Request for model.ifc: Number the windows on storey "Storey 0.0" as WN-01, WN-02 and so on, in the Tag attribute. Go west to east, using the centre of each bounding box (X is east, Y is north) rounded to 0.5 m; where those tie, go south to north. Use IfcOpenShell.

First a look at what the model holds.

```python
import ifcopenshell
import ifcopenshell.util.element
import ifcopenshell.util.placement

model = ifcopenshell.open("model.ifc")
print(model.schema)
storey = next(s for s in model.by_type("IfcBuildingStorey") if s.Name == "Storey 0.0")
windows = [e for e in ifcopenshell.util.element.get_decomposition(storey) if e.is_a("IfcWindow")]
for e in sorted(windows, key=lambda e: e.id()):
    origin = ifcopenshell.util.placement.get_local_placement(e.ObjectPlacement)[:3, 3]
    print(e.id(), e.Tag, e.Name, origin.round(2) + 0.0, sep=" | ")
```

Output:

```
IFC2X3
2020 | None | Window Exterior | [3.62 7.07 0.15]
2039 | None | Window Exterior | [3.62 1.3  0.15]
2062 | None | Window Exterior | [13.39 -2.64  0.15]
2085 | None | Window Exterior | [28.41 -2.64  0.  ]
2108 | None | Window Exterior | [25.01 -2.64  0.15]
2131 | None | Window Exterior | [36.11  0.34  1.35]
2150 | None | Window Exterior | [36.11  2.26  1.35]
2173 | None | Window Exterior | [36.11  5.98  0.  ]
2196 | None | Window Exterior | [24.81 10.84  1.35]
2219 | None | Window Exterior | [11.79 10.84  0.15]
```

```python
import ifcopenshell
import ifcopenshell.geom
import ifcopenshell.util.element
import ifcopenshell.util.shape

model = ifcopenshell.open("model.ifc")
settings = ifcopenshell.geom.settings()
settings.set("use-world-coords", True)


def centre(element):
    shape = ifcopenshell.geom.create_shape(settings, element)
    return ifcopenshell.util.shape.get_bbox_centroid(shape.geometry)


storey = next(s for s in model.by_type("IfcBuildingStorey") if s.Name == "Storey 0.0")
windows = [e for e in ifcopenshell.util.element.get_decomposition(storey) if e.is_a("IfcWindow")]

# Insertion points can sit at a corner or the storey origin, so sort by the geometry (in metres).
centres = {e: centre(e) for e in windows}
windows.sort(key=lambda e: (round(centres[e][0] / 0.5), centres[e][1]))

for i, e in enumerate(windows, start=1):
    number = f"WN-{i:02d}"
    e.Tag = number
    print(e.id(), number)

model.write("model_edited.ifc")
```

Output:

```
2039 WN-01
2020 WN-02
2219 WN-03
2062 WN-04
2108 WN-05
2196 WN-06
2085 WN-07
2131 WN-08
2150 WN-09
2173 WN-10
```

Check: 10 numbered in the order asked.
